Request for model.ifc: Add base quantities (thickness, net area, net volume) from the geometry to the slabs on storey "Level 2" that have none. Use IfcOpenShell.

First a look at what the model holds.

```python
import ifcopenshell
import ifcopenshell.util.element
import ifcopenshell.util.unit

model = ifcopenshell.open("model.ifc")
print(model.schema)
for unit_type in ("LENGTHUNIT", "AREAUNIT", "VOLUMEUNIT"):
    print(unit_type, ifcopenshell.util.unit.calculate_unit_scale(model, unit_type))
storey = next(s for s in model.by_type("IfcBuildingStorey") if s.Name == "Level 2")
slabs = [e for e in ifcopenshell.util.element.get_decomposition(storey) if e.is_a("IfcSlab")]
for e in sorted(slabs, key=lambda e: e.id()):
    print(e.id(), e.is_a(), e.Name, list(ifcopenshell.util.element.get_psets(e, qtos_only=True)), sep=" | ")
```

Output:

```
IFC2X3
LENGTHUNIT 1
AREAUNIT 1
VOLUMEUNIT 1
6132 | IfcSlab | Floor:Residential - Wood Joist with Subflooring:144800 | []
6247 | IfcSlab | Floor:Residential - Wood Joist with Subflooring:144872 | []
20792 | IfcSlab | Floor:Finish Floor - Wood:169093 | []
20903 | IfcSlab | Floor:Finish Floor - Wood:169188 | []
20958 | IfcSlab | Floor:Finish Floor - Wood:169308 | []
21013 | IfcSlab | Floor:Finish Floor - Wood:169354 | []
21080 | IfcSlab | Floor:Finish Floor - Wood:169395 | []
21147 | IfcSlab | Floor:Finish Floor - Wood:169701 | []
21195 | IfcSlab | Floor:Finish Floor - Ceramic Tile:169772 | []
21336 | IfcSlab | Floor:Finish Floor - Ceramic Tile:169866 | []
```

```python
import ifcopenshell
import ifcopenshell.api.pset
import ifcopenshell.geom
import ifcopenshell.util.element
import ifcopenshell.util.shape
import ifcopenshell.util.unit

model = ifcopenshell.open("model.ifc")
unit_scale = ifcopenshell.util.unit.calculate_unit_scale(model)
area_scale = ifcopenshell.util.unit.calculate_unit_scale(model, "AREAUNIT")
volume_scale = ifcopenshell.util.unit.calculate_unit_scale(model, "VOLUMEUNIT")
settings = ifcopenshell.geom.settings()

storey = next(s for s in model.by_type("IfcBuildingStorey") if s.Name == "Level 2")
slabs = [e for e in ifcopenshell.util.element.get_decomposition(storey) if e.is_a("IfcSlab")]

for e in sorted(slabs, key=lambda e: e.id()):
    if ifcopenshell.util.element.get_psets(e, qtos_only=True, should_inherit=False):
        continue
    # Geometry comes back in metres, in the element's own axes.
    shape = ifcopenshell.geom.create_shape(settings, e)
    values = {
        "Width": ifcopenshell.util.shape.get_z(shape.geometry) / unit_scale,
        "NetArea": ifcopenshell.util.shape.get_footprint_area(shape.geometry) / area_scale,
        "NetVolume": ifcopenshell.util.shape.get_volume(shape.geometry) / volume_scale,
    }
    qto = ifcopenshell.api.pset.add_qto(model, product=e, name="BaseQuantities")
    ifcopenshell.api.pset.edit_qto(model, qto=qto, properties=values)
    print(e.id(), {k: round(v, 3) for k, v in values.items()})

model.write("model_edited.ifc")
```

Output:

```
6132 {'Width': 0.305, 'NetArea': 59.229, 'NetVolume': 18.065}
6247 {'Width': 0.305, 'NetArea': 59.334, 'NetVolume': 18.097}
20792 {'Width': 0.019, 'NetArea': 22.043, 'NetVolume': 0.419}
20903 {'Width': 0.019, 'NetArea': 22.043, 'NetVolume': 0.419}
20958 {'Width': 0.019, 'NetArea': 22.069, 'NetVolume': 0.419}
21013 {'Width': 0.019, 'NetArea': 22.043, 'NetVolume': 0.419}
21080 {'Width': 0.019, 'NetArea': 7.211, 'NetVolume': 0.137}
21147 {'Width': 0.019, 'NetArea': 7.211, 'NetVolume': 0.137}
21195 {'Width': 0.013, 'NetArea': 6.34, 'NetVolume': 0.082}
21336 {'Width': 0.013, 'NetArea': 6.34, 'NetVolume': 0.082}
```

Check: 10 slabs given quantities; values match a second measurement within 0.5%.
